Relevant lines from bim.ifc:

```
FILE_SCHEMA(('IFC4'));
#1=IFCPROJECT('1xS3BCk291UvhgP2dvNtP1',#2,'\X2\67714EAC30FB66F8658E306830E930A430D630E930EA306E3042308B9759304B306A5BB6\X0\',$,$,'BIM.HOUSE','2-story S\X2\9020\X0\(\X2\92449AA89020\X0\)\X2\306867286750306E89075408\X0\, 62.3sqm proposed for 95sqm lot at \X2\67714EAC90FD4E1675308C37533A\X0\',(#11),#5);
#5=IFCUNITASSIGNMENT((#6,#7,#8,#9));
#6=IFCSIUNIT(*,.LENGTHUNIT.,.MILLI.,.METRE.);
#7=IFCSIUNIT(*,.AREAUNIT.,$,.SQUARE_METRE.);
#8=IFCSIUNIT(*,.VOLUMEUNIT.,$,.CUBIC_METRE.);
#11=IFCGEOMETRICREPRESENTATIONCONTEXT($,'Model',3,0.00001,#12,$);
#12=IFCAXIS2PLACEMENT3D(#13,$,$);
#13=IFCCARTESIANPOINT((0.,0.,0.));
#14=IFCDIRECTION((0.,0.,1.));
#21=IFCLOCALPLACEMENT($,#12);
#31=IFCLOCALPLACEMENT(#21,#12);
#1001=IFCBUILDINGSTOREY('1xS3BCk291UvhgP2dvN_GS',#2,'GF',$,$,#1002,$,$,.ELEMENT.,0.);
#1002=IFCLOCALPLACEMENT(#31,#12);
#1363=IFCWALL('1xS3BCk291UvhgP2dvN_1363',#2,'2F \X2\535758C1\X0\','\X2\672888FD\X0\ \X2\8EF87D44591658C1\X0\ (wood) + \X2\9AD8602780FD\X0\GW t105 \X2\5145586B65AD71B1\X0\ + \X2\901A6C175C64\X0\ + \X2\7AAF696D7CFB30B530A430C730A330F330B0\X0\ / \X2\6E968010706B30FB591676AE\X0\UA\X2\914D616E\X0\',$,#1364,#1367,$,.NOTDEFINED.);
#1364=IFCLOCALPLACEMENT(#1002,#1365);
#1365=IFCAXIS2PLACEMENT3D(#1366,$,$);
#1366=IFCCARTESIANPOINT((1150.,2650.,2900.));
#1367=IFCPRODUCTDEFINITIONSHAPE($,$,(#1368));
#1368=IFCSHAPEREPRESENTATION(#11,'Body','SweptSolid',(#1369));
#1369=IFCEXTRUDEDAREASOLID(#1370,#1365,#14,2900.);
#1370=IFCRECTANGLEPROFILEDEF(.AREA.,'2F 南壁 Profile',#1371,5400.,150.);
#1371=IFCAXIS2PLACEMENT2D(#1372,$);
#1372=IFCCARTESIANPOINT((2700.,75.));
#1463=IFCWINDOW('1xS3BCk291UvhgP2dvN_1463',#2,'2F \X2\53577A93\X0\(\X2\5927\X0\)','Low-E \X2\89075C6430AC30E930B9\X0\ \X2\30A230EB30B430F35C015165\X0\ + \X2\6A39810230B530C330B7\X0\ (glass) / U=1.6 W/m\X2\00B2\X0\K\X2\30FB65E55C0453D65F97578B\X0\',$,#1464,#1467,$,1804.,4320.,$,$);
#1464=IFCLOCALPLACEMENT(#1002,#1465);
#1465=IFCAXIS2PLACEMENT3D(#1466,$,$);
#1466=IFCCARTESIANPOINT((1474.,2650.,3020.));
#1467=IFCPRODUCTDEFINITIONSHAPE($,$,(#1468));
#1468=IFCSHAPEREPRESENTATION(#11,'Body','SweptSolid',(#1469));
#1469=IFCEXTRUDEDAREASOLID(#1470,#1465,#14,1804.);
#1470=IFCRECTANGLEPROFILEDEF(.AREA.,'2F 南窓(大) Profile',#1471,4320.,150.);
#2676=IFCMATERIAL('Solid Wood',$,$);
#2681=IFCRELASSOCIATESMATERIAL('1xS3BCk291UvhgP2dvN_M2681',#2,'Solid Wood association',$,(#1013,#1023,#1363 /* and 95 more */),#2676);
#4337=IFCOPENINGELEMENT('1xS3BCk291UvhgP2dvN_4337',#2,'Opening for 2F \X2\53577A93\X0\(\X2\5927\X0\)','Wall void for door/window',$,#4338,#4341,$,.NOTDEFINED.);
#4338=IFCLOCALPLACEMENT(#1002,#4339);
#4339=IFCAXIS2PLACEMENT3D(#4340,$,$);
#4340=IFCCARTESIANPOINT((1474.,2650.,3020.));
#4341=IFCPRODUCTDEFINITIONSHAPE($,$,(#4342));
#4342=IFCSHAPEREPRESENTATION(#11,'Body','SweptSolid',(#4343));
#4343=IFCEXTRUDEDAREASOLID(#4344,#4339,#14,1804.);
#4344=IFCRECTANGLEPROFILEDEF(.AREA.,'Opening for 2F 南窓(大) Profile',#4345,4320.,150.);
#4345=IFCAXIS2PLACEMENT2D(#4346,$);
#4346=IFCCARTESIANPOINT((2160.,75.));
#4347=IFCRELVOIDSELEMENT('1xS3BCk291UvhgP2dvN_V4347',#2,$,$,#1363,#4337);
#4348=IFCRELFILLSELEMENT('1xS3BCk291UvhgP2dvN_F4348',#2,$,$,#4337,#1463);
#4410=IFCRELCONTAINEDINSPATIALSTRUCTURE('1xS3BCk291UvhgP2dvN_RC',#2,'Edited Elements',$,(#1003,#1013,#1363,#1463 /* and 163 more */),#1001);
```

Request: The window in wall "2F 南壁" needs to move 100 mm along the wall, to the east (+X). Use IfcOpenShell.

```python
import ifcopenshell
import ifcopenshell.api.geometry
import ifcopenshell.util.placement

model = ifcopenshell.open("bim.ifc")

window = model.by_guid("1xS3BCk291UvhgP2dvN_1463")
opening = window.FillsVoids[0].RelatingOpeningElement
wall = opening.VoidsElements[0].RelatingBuildingElement

wall_matrix = ifcopenshell.util.placement.get_local_placement(wall.ObjectPlacement)
shift = wall_matrix[:3, 0] * 100.0
before = ifcopenshell.util.placement.get_local_placement(window.ObjectPlacement)[:3, 3].copy()

# The window is not placed relative to its opening, so move both.
for product in (opening, window):
    matrix = ifcopenshell.util.placement.get_local_placement(product.ObjectPlacement)
    matrix[:3, 3] += shift
    ifcopenshell.api.geometry.edit_object_placement(model, product=product, matrix=matrix, is_si=False)

after = ifcopenshell.util.placement.get_local_placement(window.ObjectPlacement)[:3, 3]
print("window moved by", (after - before).round(3) + 0.0)

model.write("bim_edited.ifc")
```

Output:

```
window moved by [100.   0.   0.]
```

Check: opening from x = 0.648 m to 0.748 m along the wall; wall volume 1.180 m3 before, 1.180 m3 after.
